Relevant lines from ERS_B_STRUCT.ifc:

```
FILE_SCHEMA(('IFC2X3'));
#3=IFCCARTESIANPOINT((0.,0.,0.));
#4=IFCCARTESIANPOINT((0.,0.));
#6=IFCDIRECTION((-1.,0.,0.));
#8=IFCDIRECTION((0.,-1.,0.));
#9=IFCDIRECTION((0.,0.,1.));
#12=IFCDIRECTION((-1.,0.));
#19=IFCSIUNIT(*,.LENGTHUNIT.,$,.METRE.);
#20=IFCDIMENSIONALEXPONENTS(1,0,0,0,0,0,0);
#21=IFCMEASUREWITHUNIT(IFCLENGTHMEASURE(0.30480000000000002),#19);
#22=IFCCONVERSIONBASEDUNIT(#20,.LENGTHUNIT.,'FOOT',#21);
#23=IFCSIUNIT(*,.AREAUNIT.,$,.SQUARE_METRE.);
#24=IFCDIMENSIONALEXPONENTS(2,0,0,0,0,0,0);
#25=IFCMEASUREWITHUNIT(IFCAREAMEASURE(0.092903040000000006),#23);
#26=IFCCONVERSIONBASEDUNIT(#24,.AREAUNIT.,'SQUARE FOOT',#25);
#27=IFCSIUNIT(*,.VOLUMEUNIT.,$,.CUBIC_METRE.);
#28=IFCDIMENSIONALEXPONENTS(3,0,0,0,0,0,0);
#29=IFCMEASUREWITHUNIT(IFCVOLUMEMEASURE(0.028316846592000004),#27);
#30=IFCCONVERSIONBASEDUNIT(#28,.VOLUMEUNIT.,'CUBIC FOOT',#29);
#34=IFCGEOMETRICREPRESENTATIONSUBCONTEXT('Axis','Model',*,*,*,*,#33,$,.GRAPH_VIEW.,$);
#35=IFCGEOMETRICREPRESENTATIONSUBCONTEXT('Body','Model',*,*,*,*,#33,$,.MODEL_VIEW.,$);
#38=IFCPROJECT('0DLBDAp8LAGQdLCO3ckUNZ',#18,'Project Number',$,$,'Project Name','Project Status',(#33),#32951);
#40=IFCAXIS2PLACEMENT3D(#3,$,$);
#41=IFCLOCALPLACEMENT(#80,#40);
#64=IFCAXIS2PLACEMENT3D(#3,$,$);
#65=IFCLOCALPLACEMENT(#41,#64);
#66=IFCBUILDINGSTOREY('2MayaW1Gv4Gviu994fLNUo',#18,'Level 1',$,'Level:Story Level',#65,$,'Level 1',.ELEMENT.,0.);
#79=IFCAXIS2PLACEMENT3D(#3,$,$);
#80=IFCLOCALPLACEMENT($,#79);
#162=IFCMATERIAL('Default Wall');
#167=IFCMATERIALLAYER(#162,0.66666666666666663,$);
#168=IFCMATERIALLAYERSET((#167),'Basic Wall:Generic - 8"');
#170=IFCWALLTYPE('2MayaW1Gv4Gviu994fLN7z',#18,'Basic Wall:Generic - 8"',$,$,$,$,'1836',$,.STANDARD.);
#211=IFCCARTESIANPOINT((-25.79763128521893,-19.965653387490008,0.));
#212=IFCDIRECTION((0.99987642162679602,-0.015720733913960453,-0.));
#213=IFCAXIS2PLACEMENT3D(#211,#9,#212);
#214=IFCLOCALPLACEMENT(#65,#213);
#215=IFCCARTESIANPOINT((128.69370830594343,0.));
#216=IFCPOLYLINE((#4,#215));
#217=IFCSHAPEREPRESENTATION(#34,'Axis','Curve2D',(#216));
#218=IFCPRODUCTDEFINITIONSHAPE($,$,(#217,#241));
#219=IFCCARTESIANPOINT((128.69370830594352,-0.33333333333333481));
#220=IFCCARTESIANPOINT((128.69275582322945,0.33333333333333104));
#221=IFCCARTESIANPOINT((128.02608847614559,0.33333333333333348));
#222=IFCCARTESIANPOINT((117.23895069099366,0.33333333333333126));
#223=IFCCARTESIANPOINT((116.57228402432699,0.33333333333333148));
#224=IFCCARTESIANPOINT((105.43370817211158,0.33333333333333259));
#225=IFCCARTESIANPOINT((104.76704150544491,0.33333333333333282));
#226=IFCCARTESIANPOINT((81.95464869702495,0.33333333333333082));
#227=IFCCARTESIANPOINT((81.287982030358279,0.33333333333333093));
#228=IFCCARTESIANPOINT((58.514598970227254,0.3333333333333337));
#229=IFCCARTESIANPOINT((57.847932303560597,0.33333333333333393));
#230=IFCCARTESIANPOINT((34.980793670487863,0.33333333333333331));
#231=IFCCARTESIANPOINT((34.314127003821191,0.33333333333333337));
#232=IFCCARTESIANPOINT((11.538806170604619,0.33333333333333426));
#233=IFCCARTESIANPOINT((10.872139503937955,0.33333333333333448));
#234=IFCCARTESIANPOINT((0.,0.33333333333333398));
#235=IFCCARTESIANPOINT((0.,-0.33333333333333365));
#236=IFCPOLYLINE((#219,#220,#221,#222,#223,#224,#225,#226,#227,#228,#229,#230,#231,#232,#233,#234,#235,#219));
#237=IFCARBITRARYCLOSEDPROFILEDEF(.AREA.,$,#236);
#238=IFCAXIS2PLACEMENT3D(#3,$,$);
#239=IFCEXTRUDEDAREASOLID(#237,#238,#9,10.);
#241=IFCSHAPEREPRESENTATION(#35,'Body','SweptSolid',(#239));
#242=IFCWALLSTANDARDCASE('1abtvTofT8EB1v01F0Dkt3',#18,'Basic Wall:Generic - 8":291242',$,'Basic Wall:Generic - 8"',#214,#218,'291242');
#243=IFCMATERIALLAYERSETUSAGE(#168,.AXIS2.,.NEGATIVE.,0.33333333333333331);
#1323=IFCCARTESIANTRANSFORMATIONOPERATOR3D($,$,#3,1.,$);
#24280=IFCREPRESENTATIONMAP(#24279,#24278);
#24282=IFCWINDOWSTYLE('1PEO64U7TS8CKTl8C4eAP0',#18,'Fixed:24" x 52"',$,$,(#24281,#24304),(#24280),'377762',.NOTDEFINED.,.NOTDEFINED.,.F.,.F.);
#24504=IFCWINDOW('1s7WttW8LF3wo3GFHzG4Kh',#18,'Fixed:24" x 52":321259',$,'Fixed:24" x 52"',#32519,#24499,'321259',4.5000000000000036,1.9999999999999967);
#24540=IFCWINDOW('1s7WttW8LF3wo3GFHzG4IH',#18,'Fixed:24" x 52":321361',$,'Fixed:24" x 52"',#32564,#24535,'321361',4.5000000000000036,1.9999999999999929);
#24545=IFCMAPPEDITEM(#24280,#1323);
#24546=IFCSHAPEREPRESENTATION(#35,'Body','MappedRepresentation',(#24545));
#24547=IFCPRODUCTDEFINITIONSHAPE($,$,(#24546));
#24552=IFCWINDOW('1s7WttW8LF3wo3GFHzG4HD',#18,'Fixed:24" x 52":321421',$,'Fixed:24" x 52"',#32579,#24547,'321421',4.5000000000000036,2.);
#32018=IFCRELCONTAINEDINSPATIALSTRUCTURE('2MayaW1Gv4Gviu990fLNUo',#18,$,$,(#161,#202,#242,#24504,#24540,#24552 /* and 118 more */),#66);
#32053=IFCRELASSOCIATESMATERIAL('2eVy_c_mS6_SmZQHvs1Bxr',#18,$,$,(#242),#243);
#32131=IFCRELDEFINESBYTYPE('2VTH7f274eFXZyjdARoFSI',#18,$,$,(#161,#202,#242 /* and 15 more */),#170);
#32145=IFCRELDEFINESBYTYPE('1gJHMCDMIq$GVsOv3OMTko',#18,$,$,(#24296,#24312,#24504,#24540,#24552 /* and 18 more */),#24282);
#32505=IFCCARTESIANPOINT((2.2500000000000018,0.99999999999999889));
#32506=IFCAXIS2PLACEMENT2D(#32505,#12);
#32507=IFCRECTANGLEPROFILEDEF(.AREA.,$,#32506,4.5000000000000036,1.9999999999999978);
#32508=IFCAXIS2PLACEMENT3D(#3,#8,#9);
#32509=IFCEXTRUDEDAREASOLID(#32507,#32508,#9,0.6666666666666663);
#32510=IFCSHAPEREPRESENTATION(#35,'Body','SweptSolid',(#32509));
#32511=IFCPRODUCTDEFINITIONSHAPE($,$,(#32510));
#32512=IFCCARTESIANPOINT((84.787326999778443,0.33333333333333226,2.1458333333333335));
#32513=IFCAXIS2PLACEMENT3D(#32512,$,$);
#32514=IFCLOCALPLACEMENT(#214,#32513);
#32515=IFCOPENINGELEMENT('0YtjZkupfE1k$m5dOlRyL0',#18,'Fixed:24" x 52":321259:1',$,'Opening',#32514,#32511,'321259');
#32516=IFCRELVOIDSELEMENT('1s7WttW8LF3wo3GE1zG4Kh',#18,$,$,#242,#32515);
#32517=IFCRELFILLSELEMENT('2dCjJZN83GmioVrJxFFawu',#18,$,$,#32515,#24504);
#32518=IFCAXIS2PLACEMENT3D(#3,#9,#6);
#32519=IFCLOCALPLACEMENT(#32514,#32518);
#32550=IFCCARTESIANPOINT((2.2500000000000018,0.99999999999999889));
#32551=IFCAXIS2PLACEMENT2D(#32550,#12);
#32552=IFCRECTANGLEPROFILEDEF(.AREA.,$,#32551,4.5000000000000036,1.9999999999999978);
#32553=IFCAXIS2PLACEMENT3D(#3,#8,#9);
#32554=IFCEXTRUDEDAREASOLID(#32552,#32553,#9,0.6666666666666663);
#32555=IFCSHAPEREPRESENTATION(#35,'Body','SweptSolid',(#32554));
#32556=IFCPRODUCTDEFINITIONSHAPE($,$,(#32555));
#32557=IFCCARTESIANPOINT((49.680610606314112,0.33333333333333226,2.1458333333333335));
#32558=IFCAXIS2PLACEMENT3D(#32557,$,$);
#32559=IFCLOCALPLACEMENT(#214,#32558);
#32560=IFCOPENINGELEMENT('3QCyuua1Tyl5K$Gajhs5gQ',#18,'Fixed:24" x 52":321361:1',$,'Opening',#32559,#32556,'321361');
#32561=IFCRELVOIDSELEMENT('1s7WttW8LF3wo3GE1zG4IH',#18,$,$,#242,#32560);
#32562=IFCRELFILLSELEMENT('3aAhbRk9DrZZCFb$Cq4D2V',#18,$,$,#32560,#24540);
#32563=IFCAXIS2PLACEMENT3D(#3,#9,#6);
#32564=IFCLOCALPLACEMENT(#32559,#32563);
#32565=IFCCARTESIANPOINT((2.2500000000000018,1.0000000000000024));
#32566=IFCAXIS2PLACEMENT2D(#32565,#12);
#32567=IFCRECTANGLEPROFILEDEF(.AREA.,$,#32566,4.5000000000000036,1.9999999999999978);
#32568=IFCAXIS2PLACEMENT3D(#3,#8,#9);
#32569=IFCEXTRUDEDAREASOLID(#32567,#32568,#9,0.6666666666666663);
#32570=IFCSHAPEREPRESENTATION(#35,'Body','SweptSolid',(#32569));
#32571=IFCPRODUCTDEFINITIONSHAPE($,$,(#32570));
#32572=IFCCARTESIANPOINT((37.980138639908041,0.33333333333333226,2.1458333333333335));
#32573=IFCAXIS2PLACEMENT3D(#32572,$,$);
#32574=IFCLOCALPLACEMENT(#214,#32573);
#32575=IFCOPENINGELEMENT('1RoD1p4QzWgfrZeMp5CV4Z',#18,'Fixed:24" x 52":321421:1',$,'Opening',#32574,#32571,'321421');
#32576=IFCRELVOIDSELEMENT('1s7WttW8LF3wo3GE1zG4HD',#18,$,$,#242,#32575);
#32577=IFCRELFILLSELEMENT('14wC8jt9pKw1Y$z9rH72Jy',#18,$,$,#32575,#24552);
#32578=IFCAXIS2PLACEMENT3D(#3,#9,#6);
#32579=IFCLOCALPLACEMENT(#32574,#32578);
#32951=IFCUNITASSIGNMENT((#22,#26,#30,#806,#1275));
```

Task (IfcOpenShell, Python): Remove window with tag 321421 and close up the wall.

```python
import ifcopenshell
import ifcopenshell.api.feature
import ifcopenshell.api.root
import ifcopenshell.geom
import ifcopenshell.util.shape

model = ifcopenshell.open("ERS_B_STRUCT.ifc")
settings = ifcopenshell.geom.settings()


def volume(element):
    """Net volume in cubic metres, openings subtracted."""
    shape = ifcopenshell.geom.create_shape(settings, element)
    return ifcopenshell.util.shape.get_volume(shape.geometry)


window = model.by_guid("1s7WttW8LF3wo3GFHzG4HD")
opening = window.FillsVoids[0].RelatingOpeningElement
wall = opening.VoidsElements[0].RelatingBuildingElement
before = volume(wall)

ifcopenshell.api.root.remove_product(model, product=window)
ifcopenshell.api.feature.remove_feature(model, feature=opening)

after = volume(wall)

print(f"wall volume {before:.3f} -> {after:.3f} m3")

model.write("ERS_B_STRUCT_rev.ifc")
```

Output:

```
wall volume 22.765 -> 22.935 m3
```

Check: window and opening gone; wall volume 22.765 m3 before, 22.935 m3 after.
